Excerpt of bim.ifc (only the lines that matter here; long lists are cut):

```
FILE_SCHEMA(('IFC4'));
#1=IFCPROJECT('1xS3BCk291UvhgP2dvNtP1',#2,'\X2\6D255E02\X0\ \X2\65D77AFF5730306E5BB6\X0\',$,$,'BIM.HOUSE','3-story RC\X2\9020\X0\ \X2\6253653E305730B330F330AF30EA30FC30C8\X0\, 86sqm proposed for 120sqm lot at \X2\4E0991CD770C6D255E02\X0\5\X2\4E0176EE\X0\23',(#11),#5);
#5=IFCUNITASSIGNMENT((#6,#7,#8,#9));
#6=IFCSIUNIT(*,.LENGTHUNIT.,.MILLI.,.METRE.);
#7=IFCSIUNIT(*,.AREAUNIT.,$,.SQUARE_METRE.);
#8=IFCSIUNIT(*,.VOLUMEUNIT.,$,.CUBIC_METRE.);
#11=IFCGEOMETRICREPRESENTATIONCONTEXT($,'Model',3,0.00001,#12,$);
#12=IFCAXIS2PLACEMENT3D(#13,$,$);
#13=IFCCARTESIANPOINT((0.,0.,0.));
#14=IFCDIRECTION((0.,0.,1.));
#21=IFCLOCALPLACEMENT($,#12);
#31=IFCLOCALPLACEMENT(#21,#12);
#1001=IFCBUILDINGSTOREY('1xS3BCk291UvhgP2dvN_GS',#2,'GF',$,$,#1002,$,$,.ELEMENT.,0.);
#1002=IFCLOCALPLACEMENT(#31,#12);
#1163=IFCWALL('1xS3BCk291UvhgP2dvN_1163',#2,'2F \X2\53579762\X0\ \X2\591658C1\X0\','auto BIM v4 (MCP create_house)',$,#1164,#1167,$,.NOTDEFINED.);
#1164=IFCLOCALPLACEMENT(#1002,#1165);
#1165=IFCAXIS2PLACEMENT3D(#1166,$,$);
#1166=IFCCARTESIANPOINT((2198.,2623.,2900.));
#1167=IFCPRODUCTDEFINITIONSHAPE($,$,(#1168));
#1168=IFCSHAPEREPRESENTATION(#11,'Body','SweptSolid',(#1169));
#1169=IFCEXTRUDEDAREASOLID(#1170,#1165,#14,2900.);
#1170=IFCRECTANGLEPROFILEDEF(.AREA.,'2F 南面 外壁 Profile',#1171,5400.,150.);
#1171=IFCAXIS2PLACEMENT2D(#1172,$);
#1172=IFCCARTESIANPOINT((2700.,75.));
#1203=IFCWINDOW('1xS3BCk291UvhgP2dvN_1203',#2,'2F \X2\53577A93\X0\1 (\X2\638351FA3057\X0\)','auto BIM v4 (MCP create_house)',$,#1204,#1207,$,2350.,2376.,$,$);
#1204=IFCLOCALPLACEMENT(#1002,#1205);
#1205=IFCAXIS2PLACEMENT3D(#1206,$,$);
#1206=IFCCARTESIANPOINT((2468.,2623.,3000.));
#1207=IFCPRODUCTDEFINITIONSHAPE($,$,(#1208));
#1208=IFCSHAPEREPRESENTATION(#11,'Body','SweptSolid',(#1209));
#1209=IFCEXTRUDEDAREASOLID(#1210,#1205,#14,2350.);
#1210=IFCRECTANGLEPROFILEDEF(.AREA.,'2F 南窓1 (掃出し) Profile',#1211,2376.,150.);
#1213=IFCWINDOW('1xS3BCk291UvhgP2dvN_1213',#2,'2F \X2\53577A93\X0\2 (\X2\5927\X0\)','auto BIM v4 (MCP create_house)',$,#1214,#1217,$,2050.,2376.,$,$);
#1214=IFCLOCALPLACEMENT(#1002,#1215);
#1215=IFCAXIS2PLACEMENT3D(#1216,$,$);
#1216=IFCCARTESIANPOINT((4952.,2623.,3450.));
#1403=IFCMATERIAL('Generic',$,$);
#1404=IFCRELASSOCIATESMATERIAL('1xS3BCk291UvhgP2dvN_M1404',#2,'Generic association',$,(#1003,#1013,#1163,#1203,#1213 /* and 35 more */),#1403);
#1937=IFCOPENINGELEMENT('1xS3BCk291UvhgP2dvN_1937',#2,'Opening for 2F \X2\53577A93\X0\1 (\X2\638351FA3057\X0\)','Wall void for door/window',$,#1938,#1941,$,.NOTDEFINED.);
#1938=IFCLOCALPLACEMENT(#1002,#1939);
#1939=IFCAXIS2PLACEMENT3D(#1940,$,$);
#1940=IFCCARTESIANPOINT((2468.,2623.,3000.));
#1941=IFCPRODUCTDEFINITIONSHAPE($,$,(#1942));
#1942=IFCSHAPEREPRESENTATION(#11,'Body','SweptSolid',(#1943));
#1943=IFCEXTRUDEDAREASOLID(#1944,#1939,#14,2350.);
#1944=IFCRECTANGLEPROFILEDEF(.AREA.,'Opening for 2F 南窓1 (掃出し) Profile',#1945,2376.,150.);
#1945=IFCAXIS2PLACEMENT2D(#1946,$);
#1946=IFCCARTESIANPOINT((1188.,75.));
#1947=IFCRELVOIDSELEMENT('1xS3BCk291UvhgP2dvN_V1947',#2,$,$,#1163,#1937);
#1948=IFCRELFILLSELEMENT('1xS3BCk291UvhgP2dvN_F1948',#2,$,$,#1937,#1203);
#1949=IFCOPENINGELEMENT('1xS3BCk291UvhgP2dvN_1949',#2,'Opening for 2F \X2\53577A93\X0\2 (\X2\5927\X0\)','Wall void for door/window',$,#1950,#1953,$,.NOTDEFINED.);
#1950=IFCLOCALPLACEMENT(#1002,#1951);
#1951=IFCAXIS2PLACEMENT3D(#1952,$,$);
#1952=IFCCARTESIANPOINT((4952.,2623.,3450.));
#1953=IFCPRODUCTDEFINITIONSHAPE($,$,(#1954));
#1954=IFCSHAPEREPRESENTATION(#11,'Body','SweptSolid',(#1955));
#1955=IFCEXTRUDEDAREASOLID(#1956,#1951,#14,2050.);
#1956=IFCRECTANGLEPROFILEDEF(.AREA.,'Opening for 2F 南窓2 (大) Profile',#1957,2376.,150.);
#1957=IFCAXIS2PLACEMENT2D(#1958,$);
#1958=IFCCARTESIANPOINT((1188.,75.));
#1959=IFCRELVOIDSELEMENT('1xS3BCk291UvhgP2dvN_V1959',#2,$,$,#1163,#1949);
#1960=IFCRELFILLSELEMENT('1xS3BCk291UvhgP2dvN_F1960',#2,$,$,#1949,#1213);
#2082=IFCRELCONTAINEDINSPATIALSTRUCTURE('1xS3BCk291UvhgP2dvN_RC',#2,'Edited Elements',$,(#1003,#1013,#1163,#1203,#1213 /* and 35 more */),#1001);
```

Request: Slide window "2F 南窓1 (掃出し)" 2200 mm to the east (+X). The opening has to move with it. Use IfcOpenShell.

```python
import ifcopenshell
import ifcopenshell.api.geometry
import ifcopenshell.util.placement

model = ifcopenshell.open("bim.ifc")

window = model.by_guid("1xS3BCk291UvhgP2dvN_1203")
opening = window.FillsVoids[0].RelatingOpeningElement
wall = opening.VoidsElements[0].RelatingBuildingElement

wall_matrix = ifcopenshell.util.placement.get_local_placement(wall.ObjectPlacement)
shift = wall_matrix[:3, 0] * 2200.0
before = ifcopenshell.util.placement.get_local_placement(window.ObjectPlacement)[:3, 3].copy()

# The window is not placed relative to its opening, so move both.
for product in (opening, window):
    matrix = ifcopenshell.util.placement.get_local_placement(product.ObjectPlacement)
    matrix[:3, 3] += shift
    ifcopenshell.api.geometry.edit_object_placement(model, product=product, matrix=matrix, is_si=False)

after = ifcopenshell.util.placement.get_local_placement(window.ObjectPlacement)[:3, 3]
print("window moved by", (after - before).round(3) + 0.0)

model.write("bim_rev.ifc")
```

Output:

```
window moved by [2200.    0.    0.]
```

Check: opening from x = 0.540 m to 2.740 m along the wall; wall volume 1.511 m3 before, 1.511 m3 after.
